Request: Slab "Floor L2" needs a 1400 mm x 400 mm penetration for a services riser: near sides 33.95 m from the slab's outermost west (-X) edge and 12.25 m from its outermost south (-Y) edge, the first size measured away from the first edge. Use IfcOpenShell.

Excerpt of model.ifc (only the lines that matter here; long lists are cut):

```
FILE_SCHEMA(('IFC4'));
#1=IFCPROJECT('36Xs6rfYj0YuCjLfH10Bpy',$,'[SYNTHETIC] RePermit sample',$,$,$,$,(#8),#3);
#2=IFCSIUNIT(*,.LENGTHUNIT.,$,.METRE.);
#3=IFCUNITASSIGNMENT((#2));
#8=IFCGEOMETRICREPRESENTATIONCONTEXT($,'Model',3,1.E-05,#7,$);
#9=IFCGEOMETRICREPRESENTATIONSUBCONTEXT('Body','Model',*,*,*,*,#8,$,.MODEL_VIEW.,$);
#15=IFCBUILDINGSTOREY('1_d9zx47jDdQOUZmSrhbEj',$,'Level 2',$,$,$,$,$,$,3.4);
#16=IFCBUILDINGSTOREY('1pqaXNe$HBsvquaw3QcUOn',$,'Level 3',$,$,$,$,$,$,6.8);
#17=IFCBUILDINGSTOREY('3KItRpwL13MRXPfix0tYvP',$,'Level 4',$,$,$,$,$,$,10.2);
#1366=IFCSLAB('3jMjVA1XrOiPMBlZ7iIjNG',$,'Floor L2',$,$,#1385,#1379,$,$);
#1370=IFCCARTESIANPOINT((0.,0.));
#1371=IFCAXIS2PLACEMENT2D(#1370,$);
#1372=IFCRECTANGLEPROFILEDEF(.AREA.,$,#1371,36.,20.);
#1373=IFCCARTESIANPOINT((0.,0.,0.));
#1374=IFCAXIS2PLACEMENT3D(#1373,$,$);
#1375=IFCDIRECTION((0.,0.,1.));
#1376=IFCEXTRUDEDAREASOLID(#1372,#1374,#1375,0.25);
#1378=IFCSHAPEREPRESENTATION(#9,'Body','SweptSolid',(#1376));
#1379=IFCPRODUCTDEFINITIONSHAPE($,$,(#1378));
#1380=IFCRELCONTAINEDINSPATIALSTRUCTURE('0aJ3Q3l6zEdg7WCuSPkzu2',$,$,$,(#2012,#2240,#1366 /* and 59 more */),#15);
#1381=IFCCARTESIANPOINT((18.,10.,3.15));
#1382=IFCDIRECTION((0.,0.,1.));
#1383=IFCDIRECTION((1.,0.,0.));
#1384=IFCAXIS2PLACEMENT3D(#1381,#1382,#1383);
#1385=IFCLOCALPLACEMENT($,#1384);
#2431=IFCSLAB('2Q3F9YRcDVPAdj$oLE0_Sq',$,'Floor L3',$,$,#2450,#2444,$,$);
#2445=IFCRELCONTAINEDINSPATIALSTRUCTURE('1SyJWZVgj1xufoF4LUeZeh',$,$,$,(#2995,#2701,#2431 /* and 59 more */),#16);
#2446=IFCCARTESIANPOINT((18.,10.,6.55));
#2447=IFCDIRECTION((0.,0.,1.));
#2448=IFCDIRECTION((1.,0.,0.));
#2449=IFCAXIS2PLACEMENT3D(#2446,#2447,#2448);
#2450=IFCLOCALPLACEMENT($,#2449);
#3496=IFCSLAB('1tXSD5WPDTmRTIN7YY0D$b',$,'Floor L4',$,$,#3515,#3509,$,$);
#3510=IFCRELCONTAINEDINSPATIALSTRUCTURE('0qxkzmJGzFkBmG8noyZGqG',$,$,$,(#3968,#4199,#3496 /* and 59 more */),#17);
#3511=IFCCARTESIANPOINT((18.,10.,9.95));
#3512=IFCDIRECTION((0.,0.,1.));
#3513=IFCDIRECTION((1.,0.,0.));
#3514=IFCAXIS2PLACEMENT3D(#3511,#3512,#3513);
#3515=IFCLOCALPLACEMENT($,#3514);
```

```python
import numpy as np
import ifcopenshell
import ifcopenshell.api.feature
import ifcopenshell.api.geometry
import ifcopenshell.api.root
import ifcopenshell.geom
import ifcopenshell.util.placement
import ifcopenshell.util.representation
import ifcopenshell.util.shape
import ifcopenshell.util.unit

model = ifcopenshell.open("model.ifc")
unit_scale = ifcopenshell.util.unit.calculate_unit_scale(model)
settings = ifcopenshell.geom.settings()


def volume(element):
    """Net volume in cubic metres, openings subtracted."""
    shape = ifcopenshell.geom.create_shape(settings, element)
    return ifcopenshell.util.shape.get_volume(shape.geometry)


slab = model.by_id(1366)
before = volume(slab)

# Extent in the slab's own axes, in metres. The edges named are its -X and -Y sides.
slab_shape = ifcopenshell.geom.create_shape(settings, slab)
vertices = ifcopenshell.util.shape.get_vertices(slab_shape.geometry)
x_min, y_min, bottom = vertices.min(axis=0)
top = vertices[:, 2].max()

opening = ifcopenshell.api.root.create_entity(model, ifc_class="IfcOpeningElement", name="Services riser opening", predefined_type="OPENING")
context = ifcopenshell.util.representation.get_context(model, "Model", "Body", "MODEL_VIEW")
width, depth = 1.4, 0.4
outline = [(0.0, 0.0), (width, 0.0), (width, depth), (0.0, depth), (0.0, 0.0)]
# Overshoot both faces by 50 mm so the cut is clean.
shape = ifcopenshell.api.geometry.add_slab_representation(
    model, context=context, depth=top - bottom + 0.1, polyline=outline
)
ifcopenshell.api.geometry.assign_representation(model, product=opening, representation=shape)

matrix = ifcopenshell.util.placement.get_local_placement(slab.ObjectPlacement)
matrix[:, 3] = matrix @ np.append(np.array([x_min + 33.95, y_min + 12.25, bottom - 0.05]) / unit_scale, 1.0)
ifcopenshell.api.geometry.edit_object_placement(model, product=opening, matrix=matrix, is_si=False)
ifcopenshell.api.feature.add_feature(model, feature=opening, element=slab)

after = volume(slab)

print(f"slab volume {before:.3f} -> {after:.3f} m3")

model.write("model_edited.ifc")
```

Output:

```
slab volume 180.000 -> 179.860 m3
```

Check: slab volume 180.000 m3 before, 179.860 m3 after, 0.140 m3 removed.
